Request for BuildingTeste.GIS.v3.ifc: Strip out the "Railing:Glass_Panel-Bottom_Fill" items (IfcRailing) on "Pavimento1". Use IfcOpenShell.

First a look at what the model holds.

```python
import ifcopenshell
import ifcopenshell.util.element

model = ifcopenshell.open("BuildingTeste.GIS.v3.ifc")
print(model.schema)
storey = next(s for s in model.by_type("IfcBuildingStorey") if s.Name == "Pavimento1")
railings = [e for e in ifcopenshell.util.element.get_decomposition(storey) if e.is_a("IfcRailing")]
seen = {}
for e in railings:
    element_type = ifcopenshell.util.element.get_type(e)
    name = element_type.Name if element_type not in (None, e) else None
    seen[name] = seen.get(name, 0) + 1
for name, count in sorted(seen.items(), key=str):
    print(count, "x", name)
```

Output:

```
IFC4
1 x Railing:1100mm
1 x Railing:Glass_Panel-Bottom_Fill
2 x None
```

```python
import ifcopenshell
import ifcopenshell.api.root
import ifcopenshell.util.element

model = ifcopenshell.open("BuildingTeste.GIS.v3.ifc")

storey = next(s for s in model.by_type("IfcBuildingStorey") if s.Name == "Pavimento1")
railings = [e for e in ifcopenshell.util.element.get_decomposition(storey) if e.is_a("IfcRailing")]
targets = [e for e in railings if (t := ifcopenshell.util.element.get_type(e)) not in (None, e) and t.Name == "Railing:Glass_Panel-Bottom_Fill"]

for e in targets:
    ifcopenshell.api.root.remove_product(model, product=e)
print(len(targets), "removed")

model.write("BuildingTeste.GIS.v3-out.ifc")
```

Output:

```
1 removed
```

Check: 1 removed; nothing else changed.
